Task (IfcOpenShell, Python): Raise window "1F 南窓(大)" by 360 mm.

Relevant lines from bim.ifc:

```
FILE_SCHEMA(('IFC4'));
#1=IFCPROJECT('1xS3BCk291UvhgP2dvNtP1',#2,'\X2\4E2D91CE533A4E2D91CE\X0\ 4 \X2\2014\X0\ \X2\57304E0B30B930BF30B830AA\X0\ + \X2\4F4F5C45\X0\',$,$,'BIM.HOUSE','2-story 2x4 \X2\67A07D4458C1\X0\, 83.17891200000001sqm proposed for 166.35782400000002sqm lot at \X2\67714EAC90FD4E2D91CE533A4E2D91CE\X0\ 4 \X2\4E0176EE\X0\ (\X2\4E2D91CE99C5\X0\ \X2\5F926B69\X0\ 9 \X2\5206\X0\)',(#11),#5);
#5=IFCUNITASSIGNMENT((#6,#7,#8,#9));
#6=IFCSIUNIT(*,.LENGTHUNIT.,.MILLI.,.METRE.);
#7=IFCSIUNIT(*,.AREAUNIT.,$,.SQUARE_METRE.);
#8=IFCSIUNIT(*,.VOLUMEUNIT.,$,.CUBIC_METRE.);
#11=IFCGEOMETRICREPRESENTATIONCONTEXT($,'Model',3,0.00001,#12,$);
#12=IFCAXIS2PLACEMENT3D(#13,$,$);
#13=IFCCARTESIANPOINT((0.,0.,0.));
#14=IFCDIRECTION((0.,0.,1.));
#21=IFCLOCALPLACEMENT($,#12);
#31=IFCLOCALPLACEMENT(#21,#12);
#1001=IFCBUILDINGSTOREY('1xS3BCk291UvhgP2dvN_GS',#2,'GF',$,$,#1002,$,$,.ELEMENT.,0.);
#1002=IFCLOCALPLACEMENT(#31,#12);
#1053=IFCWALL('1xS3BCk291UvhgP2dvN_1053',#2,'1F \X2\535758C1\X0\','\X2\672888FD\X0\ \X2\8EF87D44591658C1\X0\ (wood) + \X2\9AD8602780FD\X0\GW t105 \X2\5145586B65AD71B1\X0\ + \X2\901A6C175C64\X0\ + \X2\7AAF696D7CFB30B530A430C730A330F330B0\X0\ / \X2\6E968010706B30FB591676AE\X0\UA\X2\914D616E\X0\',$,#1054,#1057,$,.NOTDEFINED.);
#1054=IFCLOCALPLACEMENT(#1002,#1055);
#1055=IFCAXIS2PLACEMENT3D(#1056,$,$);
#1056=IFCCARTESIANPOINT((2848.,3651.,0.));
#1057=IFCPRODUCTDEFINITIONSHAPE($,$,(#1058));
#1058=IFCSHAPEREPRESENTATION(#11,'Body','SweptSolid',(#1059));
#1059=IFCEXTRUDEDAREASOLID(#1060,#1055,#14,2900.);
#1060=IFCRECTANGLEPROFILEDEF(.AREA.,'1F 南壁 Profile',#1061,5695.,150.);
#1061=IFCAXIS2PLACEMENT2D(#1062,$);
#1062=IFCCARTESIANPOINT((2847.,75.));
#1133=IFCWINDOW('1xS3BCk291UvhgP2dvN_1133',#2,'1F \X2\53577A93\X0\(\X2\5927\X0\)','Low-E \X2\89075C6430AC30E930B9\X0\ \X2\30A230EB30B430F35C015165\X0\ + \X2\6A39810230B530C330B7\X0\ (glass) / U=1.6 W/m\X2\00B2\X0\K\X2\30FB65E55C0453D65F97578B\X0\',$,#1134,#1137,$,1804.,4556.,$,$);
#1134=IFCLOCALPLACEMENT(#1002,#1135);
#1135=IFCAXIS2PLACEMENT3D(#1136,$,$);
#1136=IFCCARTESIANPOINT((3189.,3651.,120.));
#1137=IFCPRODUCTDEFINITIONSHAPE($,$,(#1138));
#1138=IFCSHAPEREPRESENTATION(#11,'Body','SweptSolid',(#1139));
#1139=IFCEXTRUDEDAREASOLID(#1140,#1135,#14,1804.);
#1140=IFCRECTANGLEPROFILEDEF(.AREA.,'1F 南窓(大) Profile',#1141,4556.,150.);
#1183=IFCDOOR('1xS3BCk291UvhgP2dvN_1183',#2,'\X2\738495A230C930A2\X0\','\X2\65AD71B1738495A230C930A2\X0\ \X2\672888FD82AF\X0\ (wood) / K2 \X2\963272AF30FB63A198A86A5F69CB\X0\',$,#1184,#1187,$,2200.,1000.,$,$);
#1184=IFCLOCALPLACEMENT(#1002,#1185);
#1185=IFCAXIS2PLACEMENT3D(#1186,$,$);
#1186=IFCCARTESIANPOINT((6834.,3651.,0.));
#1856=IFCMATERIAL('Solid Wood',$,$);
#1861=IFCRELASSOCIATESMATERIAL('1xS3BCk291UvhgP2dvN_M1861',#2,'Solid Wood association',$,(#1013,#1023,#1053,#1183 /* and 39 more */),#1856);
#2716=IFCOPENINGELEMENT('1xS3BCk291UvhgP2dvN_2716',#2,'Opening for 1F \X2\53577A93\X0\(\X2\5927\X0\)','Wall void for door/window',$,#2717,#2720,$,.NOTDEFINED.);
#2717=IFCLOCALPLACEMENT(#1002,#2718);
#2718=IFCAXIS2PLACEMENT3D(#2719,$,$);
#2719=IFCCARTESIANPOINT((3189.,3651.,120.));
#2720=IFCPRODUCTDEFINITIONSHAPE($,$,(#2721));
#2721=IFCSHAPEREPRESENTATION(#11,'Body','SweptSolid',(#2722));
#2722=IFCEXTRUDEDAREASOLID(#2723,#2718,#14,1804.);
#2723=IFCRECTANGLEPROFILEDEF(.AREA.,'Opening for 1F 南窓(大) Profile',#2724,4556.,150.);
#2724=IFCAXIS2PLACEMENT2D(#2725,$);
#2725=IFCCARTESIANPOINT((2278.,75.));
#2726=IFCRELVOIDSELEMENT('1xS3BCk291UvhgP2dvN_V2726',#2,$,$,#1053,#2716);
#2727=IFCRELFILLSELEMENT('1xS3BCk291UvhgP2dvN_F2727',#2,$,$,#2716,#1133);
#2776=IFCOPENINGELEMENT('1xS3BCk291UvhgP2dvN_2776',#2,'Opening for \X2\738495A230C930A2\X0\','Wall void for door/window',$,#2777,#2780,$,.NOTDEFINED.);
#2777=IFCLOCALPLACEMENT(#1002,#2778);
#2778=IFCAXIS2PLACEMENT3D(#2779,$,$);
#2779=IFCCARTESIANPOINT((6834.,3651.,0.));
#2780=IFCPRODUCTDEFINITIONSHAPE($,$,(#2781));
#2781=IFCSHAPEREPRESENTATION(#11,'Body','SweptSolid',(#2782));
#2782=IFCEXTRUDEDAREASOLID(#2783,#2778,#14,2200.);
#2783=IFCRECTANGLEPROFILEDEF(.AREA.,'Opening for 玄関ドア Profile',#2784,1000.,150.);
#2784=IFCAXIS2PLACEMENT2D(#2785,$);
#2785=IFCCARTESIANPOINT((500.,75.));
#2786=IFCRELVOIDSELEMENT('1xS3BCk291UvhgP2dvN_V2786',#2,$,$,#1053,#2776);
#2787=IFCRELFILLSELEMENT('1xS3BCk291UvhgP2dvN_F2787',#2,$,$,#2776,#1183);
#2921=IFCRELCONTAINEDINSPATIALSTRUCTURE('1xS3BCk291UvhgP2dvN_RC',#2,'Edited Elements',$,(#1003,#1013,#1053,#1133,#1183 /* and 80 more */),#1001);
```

```python
import numpy as np
import ifcopenshell
import ifcopenshell.api.geometry
import ifcopenshell.util.placement
import ifcopenshell.util.unit

model = ifcopenshell.open("bim.ifc")
unit_scale = ifcopenshell.util.unit.calculate_unit_scale(model)

window = model.by_guid("1xS3BCk291UvhgP2dvN_1133")
opening = window.FillsVoids[0].RelatingOpeningElement
dz = 0.36 / unit_scale

shift = np.array([0.0, 0.0, dz])
# The window is not placed relative to its opening, so move both.
for product in (opening, window):
    matrix = ifcopenshell.util.placement.get_local_placement(product.ObjectPlacement)
    matrix[:3, 3] += shift
    ifcopenshell.api.geometry.edit_object_placement(model, product=product, matrix=matrix, is_si=False)

print(f"moved by {dz * unit_scale:+.3f} m")

model.write("bim_rev.ifc")
```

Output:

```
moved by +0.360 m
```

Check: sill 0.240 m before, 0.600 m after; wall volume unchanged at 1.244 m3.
